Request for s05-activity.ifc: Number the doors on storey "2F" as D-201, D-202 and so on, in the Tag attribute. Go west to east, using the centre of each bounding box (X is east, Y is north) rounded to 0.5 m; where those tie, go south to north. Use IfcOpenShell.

First a look at what the model holds.

```python
import ifcopenshell
import ifcopenshell.util.element
import ifcopenshell.util.placement

model = ifcopenshell.open("s05-activity.ifc")
print(model.schema)
storey = next(s for s in model.by_type("IfcBuildingStorey") if s.Name == "2F")
doors = [e for e in ifcopenshell.util.element.get_decomposition(storey) if e.is_a("IfcDoor")]
for e in sorted(doors, key=lambda e: e.id()):
    origin = ifcopenshell.util.placement.get_local_placement(e.ObjectPlacement)[:3, 3]
    print(e.id(), e.Tag, e.Name, origin.round(2) + 0.0, sep=" | ")
```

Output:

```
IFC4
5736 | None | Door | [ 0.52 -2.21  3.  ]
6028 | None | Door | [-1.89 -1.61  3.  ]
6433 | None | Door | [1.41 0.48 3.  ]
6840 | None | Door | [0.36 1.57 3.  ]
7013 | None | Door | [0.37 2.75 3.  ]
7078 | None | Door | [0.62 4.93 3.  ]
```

```python
import ifcopenshell
import ifcopenshell.geom
import ifcopenshell.util.element
import ifcopenshell.util.shape

model = ifcopenshell.open("s05-activity.ifc")
settings = ifcopenshell.geom.settings()
settings.set("use-world-coords", True)


def centre(element):
    shape = ifcopenshell.geom.create_shape(settings, element)
    return ifcopenshell.util.shape.get_bbox_centroid(shape.geometry)


storey = next(s for s in model.by_type("IfcBuildingStorey") if s.Name == "2F")
doors = [e for e in ifcopenshell.util.element.get_decomposition(storey) if e.is_a("IfcDoor")]

# Insertion points can sit at a corner or the storey origin, so sort by the geometry (in metres).
centres = {e: centre(e) for e in doors}
doors.sort(key=lambda e: (round(centres[e][0] / 0.5), centres[e][1]))

for i, e in enumerate(doors, start=1):
    number = f"D-2{i:02d}"
    e.Tag = number
    print(e.id(), number)

model.write("s05-activity-out.ifc")
```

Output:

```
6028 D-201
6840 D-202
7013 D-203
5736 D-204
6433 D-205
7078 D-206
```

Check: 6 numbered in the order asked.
